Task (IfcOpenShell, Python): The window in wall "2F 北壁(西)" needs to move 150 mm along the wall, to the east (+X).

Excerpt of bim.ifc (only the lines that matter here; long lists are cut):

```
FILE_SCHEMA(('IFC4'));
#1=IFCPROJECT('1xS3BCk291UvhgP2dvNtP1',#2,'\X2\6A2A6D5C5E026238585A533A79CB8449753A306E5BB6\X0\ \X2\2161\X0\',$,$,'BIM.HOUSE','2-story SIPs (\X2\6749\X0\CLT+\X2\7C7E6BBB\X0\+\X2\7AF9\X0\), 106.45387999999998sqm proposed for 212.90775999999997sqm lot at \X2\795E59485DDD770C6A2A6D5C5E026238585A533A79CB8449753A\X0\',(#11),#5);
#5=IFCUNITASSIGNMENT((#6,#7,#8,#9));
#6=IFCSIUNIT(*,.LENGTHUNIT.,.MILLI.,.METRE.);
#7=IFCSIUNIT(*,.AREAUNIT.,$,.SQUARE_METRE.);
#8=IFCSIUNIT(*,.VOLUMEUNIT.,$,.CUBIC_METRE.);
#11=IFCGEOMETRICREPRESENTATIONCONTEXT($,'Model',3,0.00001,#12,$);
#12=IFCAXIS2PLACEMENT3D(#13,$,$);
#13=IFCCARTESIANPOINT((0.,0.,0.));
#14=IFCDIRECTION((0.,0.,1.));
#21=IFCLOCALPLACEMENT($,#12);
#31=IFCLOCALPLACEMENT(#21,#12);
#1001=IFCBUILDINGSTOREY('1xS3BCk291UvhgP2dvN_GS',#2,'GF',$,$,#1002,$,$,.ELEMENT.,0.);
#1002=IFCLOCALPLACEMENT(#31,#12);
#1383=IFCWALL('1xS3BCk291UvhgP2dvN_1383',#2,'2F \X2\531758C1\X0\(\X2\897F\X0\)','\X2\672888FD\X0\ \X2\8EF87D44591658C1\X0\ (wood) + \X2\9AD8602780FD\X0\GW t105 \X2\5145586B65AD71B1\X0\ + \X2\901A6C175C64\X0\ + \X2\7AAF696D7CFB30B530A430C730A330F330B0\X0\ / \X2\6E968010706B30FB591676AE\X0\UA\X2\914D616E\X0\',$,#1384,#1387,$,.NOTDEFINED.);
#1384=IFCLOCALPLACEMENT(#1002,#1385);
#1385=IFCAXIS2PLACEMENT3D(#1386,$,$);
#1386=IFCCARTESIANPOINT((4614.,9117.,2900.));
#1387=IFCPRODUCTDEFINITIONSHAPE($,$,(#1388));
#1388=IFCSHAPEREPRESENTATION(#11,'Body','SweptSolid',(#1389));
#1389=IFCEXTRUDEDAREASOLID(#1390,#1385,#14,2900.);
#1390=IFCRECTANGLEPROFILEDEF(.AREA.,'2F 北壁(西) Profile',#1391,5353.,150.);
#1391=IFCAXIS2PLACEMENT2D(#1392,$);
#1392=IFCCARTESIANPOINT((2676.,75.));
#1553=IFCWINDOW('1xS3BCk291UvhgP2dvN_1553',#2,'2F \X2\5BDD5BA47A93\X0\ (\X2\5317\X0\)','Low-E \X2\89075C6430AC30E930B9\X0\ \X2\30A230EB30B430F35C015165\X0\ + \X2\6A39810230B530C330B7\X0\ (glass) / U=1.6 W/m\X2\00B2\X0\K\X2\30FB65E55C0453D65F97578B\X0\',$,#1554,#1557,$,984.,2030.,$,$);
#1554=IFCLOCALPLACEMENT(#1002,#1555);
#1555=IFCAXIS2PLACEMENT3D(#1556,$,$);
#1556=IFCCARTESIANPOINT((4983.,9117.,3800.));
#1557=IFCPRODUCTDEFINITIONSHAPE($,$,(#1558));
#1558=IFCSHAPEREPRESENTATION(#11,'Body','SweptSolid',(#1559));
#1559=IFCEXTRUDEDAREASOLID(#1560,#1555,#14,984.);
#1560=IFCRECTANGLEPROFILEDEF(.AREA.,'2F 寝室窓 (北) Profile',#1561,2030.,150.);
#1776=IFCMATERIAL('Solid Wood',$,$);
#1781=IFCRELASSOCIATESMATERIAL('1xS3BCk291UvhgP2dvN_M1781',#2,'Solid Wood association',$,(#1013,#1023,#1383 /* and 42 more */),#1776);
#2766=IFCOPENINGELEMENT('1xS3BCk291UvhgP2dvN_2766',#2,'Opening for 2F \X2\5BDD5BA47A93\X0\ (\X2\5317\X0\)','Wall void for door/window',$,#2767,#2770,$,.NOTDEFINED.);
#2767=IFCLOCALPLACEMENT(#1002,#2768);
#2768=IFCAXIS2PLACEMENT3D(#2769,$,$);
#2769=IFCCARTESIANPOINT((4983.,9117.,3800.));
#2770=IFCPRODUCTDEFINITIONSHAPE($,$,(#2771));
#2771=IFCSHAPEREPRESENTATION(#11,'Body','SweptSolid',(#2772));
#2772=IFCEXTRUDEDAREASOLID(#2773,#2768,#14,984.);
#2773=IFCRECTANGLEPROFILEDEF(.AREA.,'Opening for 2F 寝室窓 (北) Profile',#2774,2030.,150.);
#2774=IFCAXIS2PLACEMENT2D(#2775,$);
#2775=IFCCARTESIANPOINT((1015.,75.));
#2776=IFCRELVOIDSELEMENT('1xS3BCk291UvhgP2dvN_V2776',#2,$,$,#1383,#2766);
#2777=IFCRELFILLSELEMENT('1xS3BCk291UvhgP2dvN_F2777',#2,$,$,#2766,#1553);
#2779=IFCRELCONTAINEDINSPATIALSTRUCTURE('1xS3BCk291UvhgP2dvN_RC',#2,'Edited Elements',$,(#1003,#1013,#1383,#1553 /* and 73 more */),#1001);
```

```python
import ifcopenshell
import ifcopenshell.api.geometry
import ifcopenshell.util.placement

model = ifcopenshell.open("bim.ifc")

window = model.by_guid("1xS3BCk291UvhgP2dvN_1553")
opening = window.FillsVoids[0].RelatingOpeningElement
wall = opening.VoidsElements[0].RelatingBuildingElement

wall_matrix = ifcopenshell.util.placement.get_local_placement(wall.ObjectPlacement)
shift = wall_matrix[:3, 0] * 150.0
before = ifcopenshell.util.placement.get_local_placement(window.ObjectPlacement)[:3, 3].copy()

# The window is not placed relative to its opening, so move both.
for product in (opening, window):
    matrix = ifcopenshell.util.placement.get_local_placement(product.ObjectPlacement)
    matrix[:3, 3] += shift
    ifcopenshell.api.geometry.edit_object_placement(model, product=product, matrix=matrix, is_si=False)

after = ifcopenshell.util.placement.get_local_placement(window.ObjectPlacement)[:3, 3]
print("window moved by", (after - before).round(3) + 0.0)

model.write("bim-out.ifc")
```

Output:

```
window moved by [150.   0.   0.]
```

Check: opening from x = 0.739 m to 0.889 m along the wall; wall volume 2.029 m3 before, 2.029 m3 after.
